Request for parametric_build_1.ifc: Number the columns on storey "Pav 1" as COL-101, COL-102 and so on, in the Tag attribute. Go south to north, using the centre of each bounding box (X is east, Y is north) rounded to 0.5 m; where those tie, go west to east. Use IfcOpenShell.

First a look at what the model holds.

```python
import ifcopenshell
import ifcopenshell.util.element
import ifcopenshell.util.placement

model = ifcopenshell.open("parametric_build_1.ifc")
print(model.schema)
storey = next(s for s in model.by_type("IfcBuildingStorey") if s.Name == "Pav 1")
columns = [e for e in ifcopenshell.util.element.get_decomposition(storey) if e.is_a("IfcColumn")]
for e in sorted(columns, key=lambda e: e.id()):
    origin = ifcopenshell.util.placement.get_local_placement(e.ObjectPlacement)[:3, 3]
    print(e.id(), e.Tag, e.Name, origin.round(2) + 0.0, sep=" | ")
```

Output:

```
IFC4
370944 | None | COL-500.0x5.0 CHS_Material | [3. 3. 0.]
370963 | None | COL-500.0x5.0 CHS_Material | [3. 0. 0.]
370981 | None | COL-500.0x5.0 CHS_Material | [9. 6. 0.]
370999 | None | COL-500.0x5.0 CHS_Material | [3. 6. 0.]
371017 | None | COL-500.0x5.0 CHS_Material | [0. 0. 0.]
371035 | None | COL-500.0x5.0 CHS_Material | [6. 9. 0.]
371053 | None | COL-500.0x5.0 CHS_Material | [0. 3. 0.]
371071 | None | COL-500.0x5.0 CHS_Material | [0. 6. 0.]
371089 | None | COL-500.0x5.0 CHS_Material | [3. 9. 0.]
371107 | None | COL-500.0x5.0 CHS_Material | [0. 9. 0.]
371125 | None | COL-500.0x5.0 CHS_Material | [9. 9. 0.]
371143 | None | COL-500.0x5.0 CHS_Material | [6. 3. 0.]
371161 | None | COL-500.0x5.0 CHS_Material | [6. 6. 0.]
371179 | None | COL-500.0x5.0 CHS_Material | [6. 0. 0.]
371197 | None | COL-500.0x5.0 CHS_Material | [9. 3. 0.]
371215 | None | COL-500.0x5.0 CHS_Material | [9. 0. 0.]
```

```python
import ifcopenshell
import ifcopenshell.geom
import ifcopenshell.util.element
import ifcopenshell.util.shape

model = ifcopenshell.open("parametric_build_1.ifc")
settings = ifcopenshell.geom.settings()
settings.set("use-world-coords", True)


def centre(element):
    shape = ifcopenshell.geom.create_shape(settings, element)
    return ifcopenshell.util.shape.get_bbox_centroid(shape.geometry)


storey = next(s for s in model.by_type("IfcBuildingStorey") if s.Name == "Pav 1")
columns = [e for e in ifcopenshell.util.element.get_decomposition(storey) if e.is_a("IfcColumn")]

# Insertion points can sit at a corner or the storey origin, so sort by the geometry (in metres).
centres = {e: centre(e) for e in columns}
columns.sort(key=lambda e: (round(centres[e][1] / 0.5), centres[e][0]))

for i, e in enumerate(columns, start=1):
    number = f"COL-1{i:02d}"
    e.Tag = number
    print(e.id(), number)

model.write("parametric_build_1_updated.ifc")
```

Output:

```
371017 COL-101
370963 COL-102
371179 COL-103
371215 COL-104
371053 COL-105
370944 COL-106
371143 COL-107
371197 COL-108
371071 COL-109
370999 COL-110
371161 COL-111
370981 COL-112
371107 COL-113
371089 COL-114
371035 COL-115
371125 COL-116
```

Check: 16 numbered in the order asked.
